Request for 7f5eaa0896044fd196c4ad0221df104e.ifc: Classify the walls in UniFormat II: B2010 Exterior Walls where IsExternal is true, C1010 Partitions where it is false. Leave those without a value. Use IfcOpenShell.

First a look at what the model holds.

```python
import ifcopenshell
import ifcopenshell.util.element

model = ifcopenshell.open("7f5eaa0896044fd196c4ad0221df104e.ifc")
print(model.schema)
print("classifications:", [c.Name for c in model.by_type("IfcClassification")])
values = [ifcopenshell.util.element.get_pset(e, "Pset_WallCommon", "IsExternal") for e in model.by_type("IfcWall")]
for value in (True, False, None):
    print("IsExternal", value, values.count(value))
```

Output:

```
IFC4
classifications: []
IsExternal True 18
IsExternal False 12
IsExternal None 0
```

```python
import ifcopenshell
import ifcopenshell.api.classification
import ifcopenshell.util.element

model = ifcopenshell.open("7f5eaa0896044fd196c4ad0221df104e.ifc")

system = ifcopenshell.api.classification.add_classification(model, classification="UniFormat II")

walls = model.by_type("IfcWall")
external = {e: ifcopenshell.util.element.get_pset(e, "Pset_WallCommon", "IsExternal") for e in walls}
for flag, code, name in ((True, "B2010", "Exterior Walls"), (False, "C1010", "Partitions")):
    products = [e for e in walls if external[e] is flag]
    ifcopenshell.api.classification.add_reference(
        model, products=products, classification=system, identification=code, name=name
    )
    print(code, len(products))

model.write("7f5eaa0896044fd196c4ad0221df104e_edited.ifc")
```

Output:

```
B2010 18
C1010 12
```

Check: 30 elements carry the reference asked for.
